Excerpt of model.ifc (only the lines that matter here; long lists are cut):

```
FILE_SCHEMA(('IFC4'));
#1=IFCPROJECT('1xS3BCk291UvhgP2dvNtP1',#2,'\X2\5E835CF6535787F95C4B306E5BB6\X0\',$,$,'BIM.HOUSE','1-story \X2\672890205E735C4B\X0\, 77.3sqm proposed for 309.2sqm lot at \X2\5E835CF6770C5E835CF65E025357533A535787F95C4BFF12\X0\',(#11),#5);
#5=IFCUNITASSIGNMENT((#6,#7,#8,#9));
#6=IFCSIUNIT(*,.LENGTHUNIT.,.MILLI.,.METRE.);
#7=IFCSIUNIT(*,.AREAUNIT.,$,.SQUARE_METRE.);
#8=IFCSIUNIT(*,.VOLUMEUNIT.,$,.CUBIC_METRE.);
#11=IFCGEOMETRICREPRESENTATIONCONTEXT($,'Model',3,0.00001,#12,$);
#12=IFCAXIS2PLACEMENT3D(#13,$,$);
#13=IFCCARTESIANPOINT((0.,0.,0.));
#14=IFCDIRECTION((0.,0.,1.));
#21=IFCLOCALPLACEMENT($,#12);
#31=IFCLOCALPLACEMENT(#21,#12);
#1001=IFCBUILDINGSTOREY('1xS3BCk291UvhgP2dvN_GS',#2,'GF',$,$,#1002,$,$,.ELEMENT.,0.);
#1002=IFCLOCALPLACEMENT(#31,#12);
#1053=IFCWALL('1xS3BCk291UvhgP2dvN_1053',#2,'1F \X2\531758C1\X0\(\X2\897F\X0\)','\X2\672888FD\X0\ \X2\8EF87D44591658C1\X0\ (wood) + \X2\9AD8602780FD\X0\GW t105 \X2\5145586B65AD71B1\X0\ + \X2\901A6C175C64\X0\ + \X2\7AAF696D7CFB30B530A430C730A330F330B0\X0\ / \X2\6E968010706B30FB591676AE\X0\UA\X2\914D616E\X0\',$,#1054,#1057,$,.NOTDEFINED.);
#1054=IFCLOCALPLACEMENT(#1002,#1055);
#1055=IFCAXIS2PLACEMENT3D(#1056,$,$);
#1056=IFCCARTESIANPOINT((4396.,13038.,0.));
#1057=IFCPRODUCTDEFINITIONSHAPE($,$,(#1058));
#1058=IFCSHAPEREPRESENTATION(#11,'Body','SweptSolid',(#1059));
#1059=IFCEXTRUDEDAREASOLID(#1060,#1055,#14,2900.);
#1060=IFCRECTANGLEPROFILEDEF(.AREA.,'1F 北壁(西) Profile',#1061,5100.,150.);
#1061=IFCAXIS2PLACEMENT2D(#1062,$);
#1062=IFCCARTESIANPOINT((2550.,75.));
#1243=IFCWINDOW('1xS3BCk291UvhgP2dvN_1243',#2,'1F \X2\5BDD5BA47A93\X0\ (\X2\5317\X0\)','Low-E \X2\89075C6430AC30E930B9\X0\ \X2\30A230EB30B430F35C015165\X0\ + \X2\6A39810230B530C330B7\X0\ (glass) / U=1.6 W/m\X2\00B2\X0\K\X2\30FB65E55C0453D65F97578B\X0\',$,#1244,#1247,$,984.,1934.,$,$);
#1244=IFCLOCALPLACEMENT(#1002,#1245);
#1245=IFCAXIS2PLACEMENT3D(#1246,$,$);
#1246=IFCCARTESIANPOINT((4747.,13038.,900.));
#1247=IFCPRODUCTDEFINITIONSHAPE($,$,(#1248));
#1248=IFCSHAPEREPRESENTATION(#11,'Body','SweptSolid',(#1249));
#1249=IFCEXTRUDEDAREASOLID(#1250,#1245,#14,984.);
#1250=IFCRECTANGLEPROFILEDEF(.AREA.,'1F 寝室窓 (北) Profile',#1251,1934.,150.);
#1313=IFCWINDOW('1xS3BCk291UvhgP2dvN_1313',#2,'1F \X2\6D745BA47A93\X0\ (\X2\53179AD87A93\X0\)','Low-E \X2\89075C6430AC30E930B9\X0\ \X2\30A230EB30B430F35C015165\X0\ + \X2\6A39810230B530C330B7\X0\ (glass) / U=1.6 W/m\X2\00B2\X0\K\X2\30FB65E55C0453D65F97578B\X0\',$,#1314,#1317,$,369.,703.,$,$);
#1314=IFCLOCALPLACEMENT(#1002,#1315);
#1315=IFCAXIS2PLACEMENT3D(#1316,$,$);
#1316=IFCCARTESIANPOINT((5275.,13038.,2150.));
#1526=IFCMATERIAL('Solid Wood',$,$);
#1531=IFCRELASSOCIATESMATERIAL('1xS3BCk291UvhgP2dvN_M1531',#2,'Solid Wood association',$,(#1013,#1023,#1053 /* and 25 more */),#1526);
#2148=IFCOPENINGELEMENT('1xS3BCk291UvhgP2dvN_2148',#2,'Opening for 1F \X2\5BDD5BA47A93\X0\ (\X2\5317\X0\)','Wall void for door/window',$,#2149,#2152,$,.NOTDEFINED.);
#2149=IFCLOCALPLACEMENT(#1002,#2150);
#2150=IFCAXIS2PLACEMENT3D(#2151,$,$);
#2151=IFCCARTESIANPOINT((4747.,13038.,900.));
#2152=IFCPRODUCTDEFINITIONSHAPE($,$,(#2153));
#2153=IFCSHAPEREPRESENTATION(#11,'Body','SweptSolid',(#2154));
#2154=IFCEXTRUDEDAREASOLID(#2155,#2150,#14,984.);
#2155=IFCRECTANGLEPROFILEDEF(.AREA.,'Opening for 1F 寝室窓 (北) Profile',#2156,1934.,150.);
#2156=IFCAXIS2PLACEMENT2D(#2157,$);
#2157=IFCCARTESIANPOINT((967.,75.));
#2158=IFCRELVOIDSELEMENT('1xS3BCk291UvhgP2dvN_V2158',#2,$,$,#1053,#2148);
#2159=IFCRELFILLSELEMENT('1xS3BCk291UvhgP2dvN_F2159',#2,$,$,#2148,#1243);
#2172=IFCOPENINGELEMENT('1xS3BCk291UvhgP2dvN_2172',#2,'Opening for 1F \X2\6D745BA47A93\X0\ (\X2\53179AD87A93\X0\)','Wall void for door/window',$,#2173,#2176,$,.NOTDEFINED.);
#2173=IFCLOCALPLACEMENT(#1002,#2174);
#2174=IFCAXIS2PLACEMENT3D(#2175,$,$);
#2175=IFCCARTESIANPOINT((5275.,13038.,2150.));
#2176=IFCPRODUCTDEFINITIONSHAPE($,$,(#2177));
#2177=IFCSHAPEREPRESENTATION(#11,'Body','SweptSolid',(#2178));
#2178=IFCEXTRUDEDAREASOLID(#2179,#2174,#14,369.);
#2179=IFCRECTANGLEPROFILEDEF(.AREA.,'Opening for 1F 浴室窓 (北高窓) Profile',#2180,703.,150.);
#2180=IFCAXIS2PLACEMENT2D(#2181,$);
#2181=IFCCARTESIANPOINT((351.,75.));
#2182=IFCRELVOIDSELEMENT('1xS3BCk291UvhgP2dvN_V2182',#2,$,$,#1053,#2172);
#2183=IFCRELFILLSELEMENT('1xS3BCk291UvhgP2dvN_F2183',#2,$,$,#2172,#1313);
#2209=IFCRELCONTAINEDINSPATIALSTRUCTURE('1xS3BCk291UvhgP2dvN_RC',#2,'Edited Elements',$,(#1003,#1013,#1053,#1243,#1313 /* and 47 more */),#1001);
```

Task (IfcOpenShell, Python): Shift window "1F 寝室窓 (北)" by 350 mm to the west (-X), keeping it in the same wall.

```python
import ifcopenshell
import ifcopenshell.api.geometry
import ifcopenshell.util.placement

model = ifcopenshell.open("model.ifc")

window = model.by_guid("1xS3BCk291UvhgP2dvN_1243")
opening = window.FillsVoids[0].RelatingOpeningElement
wall = opening.VoidsElements[0].RelatingBuildingElement

wall_matrix = ifcopenshell.util.placement.get_local_placement(wall.ObjectPlacement)
shift = wall_matrix[:3, 0] * -350.0
before = ifcopenshell.util.placement.get_local_placement(window.ObjectPlacement)[:3, 3].copy()

# The window is not placed relative to its opening, so move both.
for product in (opening, window):
    matrix = ifcopenshell.util.placement.get_local_placement(product.ObjectPlacement)
    matrix[:3, 3] += shift
    ifcopenshell.api.geometry.edit_object_placement(model, product=product, matrix=matrix, is_si=False)

after = ifcopenshell.util.placement.get_local_placement(window.ObjectPlacement)[:3, 3]
print("window moved by", (after - before).round(3) + 0.0)

model.write("model_v2.ifc")
```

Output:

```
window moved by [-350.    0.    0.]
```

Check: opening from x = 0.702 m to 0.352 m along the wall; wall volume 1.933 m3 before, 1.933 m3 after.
